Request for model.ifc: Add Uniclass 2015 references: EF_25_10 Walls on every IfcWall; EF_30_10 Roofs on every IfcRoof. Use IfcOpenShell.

First a look at what the model holds.

```python
import ifcopenshell

model = ifcopenshell.open("model.ifc")
print(model.schema)
print("classifications:", [c.Name for c in model.by_type("IfcClassification")])
for ifc_class in ("IfcDoor", "IfcRoof", "IfcStair", "IfcWall", "IfcWindow"):
    print(ifc_class, len(model.by_type(ifc_class)))
```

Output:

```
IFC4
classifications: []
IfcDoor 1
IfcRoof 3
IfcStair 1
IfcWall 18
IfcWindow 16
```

```python
import ifcopenshell
import ifcopenshell.api.classification

model = ifcopenshell.open("model.ifc")

system = ifcopenshell.api.classification.add_classification(model, classification="Uniclass 2015")

codes = {
    "IfcWall": ("EF_25_10", "Walls"),
    "IfcRoof": ("EF_30_10", "Roofs"),
}
for ifc_class, (code, name) in codes.items():
    products = model.by_type(ifc_class)
    ifcopenshell.api.classification.add_reference(
        model, products=products, classification=system, identification=code, name=name
    )
    print(code, len(products))

model.write("model_edited.ifc")
```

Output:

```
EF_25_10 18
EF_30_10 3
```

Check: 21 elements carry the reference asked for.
